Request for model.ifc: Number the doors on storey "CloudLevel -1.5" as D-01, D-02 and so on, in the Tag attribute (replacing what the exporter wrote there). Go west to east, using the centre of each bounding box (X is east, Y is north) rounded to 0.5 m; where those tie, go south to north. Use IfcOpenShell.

First a look at what the model holds.

```python
import ifcopenshell
import ifcopenshell.util.element
import ifcopenshell.util.placement

model = ifcopenshell.open("model.ifc")
print(model.schema)
storey = next(s for s in model.by_type("IfcBuildingStorey") if s.Name == "CloudLevel -1.5")
doors = [e for e in ifcopenshell.util.element.get_decomposition(storey) if e.is_a("IfcDoor")]
for e in sorted(doors, key=lambda e: e.id()):
    origin = ifcopenshell.util.placement.get_local_placement(e.ObjectPlacement)[:3, 3]
    print(e.id(), e.Tag, e.Name, origin.round(2) + 0.0, sep=" | ")
```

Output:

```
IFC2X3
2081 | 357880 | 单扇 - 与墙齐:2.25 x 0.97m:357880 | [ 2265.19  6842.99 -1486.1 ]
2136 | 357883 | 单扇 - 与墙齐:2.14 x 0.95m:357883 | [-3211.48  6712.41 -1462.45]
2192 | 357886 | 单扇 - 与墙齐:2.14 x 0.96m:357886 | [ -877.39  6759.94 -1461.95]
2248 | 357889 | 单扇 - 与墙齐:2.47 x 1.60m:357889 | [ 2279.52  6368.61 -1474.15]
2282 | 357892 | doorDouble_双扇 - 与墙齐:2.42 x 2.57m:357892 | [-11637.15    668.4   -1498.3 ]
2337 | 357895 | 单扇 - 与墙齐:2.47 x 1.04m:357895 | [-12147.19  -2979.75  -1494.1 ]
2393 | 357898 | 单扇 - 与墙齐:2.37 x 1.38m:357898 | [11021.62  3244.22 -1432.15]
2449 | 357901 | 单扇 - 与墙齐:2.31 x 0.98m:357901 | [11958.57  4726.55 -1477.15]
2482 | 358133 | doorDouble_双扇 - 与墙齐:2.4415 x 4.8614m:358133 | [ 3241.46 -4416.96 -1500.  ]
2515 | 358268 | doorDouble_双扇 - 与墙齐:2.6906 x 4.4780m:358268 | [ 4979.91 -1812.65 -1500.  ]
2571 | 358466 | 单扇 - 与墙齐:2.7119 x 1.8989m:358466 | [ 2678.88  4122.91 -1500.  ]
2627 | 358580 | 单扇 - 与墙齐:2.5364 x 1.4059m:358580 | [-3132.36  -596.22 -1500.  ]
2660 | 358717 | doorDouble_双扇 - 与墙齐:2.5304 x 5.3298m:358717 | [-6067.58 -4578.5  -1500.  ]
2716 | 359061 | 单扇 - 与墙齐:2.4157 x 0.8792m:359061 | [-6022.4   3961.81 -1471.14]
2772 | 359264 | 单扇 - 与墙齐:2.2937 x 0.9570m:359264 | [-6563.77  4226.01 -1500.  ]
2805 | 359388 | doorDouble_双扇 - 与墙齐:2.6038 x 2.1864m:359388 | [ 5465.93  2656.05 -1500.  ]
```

```python
import ifcopenshell
import ifcopenshell.geom
import ifcopenshell.util.element
import ifcopenshell.util.shape

model = ifcopenshell.open("model.ifc")
settings = ifcopenshell.geom.settings()
settings.set("use-world-coords", True)


def centre(element):
    shape = ifcopenshell.geom.create_shape(settings, element)
    return ifcopenshell.util.shape.get_bbox_centroid(shape.geometry)


storey = next(s for s in model.by_type("IfcBuildingStorey") if s.Name == "CloudLevel -1.5")
doors = [e for e in ifcopenshell.util.element.get_decomposition(storey) if e.is_a("IfcDoor")]

# Insertion points can sit at a corner or the storey origin, so sort by the geometry (in metres).
centres = {e: centre(e) for e in doors}
doors.sort(key=lambda e: (round(centres[e][0] / 0.5), centres[e][1]))

for i, e in enumerate(doors, start=1):
    number = f"D-{i:02d}"
    e.Tag = number
    print(e.id(), number)

model.write("model-out.ifc")
```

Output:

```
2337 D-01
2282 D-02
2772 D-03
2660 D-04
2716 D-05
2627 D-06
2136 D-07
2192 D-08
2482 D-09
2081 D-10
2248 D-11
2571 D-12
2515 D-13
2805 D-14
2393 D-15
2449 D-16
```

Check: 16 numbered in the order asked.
